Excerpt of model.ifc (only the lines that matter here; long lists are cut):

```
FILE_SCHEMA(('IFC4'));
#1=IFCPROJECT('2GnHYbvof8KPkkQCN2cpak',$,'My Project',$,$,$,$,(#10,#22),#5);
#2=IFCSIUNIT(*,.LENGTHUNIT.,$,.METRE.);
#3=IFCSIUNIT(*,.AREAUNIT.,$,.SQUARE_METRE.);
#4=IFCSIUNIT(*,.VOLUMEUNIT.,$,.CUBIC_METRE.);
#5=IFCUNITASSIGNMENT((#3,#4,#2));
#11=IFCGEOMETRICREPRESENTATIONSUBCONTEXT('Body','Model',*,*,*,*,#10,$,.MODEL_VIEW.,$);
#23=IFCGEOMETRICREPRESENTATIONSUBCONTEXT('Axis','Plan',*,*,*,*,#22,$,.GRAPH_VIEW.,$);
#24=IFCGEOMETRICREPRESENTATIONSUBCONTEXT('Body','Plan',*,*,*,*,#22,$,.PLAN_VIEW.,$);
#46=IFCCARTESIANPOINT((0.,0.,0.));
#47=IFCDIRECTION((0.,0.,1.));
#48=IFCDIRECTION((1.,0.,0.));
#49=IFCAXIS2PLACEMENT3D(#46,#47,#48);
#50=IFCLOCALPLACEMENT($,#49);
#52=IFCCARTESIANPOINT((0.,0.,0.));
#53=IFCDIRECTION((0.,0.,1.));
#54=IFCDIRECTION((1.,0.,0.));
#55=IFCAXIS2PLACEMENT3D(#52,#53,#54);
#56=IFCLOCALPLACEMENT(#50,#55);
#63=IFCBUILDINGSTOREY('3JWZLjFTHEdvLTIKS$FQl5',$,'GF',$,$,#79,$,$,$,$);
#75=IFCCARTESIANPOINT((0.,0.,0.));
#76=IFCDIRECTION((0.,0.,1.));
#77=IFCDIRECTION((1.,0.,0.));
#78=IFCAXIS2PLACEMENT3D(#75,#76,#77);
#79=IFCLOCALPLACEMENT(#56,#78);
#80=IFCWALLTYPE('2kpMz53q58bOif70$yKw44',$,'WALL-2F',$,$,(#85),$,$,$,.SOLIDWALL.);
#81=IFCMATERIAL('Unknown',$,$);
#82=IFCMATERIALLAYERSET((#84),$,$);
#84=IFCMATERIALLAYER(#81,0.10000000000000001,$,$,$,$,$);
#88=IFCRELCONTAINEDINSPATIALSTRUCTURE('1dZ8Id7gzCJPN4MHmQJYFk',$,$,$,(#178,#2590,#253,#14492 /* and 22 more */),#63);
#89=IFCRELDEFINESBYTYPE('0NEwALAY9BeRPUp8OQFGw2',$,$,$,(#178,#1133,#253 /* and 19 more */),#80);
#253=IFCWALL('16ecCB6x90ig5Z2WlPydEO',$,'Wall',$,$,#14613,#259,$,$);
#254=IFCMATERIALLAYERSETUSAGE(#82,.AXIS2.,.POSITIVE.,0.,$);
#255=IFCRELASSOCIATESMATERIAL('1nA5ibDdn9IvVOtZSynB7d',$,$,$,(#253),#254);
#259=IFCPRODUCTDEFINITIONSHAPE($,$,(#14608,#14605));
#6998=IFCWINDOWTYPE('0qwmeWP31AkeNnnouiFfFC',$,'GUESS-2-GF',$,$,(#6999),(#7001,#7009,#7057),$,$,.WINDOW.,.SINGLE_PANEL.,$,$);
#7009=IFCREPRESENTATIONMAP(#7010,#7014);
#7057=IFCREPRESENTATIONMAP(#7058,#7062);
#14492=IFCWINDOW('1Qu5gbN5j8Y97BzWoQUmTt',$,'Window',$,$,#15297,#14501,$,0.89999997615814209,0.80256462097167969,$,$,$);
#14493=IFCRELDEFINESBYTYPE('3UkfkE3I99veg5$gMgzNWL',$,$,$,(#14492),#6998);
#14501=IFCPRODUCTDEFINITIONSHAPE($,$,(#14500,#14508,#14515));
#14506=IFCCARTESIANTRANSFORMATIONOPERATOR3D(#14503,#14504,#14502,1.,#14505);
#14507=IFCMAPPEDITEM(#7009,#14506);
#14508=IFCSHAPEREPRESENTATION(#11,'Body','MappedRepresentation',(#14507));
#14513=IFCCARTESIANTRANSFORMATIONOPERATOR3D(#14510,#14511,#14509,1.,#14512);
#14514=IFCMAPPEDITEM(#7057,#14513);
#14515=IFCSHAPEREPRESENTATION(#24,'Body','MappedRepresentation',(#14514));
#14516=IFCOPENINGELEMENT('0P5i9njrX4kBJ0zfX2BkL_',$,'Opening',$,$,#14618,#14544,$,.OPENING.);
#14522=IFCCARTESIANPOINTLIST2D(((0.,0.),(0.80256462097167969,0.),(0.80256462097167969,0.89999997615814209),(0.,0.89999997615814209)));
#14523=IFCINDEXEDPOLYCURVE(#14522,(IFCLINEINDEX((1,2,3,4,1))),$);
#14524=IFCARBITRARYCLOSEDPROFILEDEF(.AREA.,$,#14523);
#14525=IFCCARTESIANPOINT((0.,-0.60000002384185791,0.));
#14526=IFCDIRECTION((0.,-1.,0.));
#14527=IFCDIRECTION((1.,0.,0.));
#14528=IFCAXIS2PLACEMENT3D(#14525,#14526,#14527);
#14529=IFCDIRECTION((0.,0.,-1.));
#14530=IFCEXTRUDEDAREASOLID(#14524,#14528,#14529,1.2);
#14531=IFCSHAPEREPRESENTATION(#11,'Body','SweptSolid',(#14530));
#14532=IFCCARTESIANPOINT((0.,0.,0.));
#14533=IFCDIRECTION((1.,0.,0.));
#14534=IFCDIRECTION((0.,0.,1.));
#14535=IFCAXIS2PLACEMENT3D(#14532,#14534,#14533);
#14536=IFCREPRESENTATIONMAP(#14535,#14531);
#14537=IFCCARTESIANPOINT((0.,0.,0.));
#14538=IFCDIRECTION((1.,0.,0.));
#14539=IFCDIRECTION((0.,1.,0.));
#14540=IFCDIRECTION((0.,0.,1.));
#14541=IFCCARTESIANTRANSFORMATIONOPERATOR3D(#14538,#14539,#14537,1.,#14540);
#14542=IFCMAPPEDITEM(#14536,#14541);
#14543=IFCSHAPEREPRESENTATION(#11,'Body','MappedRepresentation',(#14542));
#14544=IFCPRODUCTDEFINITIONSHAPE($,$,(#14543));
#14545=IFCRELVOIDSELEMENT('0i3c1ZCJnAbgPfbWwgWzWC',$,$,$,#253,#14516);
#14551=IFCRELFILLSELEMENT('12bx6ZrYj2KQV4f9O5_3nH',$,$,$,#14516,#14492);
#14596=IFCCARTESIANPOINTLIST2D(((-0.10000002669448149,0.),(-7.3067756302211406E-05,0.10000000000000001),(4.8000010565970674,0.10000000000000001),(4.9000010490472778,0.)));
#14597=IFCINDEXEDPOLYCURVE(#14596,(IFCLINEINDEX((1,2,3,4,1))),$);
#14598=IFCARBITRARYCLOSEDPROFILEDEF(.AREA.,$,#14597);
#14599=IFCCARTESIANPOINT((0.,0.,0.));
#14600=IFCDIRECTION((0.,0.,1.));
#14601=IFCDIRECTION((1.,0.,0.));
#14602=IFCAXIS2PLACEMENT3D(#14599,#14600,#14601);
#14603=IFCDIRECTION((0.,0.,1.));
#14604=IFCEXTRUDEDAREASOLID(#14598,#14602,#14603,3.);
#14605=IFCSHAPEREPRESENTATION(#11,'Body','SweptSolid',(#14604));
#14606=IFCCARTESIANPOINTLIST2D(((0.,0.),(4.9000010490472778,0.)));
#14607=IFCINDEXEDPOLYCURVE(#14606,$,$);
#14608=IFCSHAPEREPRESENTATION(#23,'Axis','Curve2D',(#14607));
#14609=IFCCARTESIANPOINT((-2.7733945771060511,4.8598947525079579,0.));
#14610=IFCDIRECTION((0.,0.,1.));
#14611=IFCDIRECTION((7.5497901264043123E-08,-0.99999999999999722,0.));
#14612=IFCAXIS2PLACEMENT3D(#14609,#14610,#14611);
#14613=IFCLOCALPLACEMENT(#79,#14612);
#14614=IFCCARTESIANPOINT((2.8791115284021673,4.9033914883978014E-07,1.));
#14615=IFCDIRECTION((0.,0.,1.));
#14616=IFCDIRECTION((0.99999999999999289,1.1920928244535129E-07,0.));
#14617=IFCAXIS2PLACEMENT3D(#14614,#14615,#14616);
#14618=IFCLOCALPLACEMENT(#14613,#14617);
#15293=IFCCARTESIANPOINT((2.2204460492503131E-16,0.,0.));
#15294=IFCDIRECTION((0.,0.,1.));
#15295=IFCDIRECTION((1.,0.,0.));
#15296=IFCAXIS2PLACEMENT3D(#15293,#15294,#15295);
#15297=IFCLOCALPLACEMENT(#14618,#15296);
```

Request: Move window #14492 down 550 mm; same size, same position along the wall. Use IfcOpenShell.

```python
import numpy as np
import ifcopenshell
import ifcopenshell.api.geometry
import ifcopenshell.util.placement
import ifcopenshell.util.unit

model = ifcopenshell.open("model.ifc")
unit_scale = ifcopenshell.util.unit.calculate_unit_scale(model)

window = model.by_guid("1Qu5gbN5j8Y97BzWoQUmTt")
opening = window.FillsVoids[0].RelatingOpeningElement
dz = -0.55 / unit_scale

shift = np.array([0.0, 0.0, dz])
# The window is placed relative to its opening, so it follows when the opening moves.
matrix = ifcopenshell.util.placement.get_local_placement(opening.ObjectPlacement)
matrix[:3, 3] += shift
ifcopenshell.api.geometry.edit_object_placement(
    model, product=opening, matrix=matrix, is_si=False, should_transform_children=True
)

print(f"moved by {dz * unit_scale:+.3f} m")

model.write("model-out.ifc")
```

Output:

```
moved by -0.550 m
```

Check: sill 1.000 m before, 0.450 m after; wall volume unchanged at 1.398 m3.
